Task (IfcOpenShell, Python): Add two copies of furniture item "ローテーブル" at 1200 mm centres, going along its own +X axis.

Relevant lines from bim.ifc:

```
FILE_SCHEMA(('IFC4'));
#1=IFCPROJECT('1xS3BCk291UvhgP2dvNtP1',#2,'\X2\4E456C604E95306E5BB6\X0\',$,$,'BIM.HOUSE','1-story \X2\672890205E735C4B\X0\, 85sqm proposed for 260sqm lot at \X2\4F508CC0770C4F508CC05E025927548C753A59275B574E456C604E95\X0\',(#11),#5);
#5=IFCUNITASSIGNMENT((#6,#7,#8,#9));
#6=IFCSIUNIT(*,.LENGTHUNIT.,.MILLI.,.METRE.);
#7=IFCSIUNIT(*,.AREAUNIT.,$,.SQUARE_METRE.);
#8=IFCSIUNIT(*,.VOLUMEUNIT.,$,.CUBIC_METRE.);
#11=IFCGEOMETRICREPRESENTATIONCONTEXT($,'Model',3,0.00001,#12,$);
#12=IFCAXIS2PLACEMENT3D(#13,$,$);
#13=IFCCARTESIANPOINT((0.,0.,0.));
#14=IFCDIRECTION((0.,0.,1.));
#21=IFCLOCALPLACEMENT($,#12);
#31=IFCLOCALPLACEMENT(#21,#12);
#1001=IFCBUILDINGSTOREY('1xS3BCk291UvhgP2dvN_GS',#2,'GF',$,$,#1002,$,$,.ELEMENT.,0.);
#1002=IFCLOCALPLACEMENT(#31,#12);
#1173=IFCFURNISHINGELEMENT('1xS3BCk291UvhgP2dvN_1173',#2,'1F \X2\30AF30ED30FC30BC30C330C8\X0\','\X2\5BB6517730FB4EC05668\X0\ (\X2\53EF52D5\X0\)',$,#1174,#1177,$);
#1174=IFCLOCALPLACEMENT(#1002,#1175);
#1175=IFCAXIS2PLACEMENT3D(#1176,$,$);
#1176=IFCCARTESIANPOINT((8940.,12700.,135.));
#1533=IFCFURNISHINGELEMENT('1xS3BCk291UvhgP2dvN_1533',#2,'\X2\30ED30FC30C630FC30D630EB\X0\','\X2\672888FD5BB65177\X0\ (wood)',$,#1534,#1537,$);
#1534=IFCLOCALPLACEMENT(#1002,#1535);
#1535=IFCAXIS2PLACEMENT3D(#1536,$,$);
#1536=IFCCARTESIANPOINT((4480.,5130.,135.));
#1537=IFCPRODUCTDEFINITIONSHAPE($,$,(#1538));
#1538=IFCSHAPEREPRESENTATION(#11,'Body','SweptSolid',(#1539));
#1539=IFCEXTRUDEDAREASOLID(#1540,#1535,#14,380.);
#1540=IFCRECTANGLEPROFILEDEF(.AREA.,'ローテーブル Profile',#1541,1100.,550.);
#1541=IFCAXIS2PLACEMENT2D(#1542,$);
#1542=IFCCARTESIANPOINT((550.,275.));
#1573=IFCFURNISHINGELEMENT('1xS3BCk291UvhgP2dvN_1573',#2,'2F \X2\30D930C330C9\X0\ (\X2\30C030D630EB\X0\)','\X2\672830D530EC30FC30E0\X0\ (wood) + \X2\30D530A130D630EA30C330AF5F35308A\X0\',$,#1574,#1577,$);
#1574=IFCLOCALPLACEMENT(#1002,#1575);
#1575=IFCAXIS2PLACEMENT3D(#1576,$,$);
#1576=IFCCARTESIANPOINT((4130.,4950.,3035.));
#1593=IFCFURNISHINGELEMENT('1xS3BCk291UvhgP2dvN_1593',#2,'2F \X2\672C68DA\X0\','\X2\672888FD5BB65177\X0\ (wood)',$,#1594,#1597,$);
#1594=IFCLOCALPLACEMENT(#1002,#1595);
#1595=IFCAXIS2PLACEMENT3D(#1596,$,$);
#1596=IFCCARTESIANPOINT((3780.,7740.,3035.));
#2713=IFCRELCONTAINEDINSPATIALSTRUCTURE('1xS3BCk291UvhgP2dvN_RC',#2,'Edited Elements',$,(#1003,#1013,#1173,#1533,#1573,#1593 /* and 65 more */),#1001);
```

```python
import ifcopenshell
import ifcopenshell.api.geometry
import ifcopenshell.api.root
import ifcopenshell.util.element
import ifcopenshell.util.placement
import ifcopenshell.util.unit

model = ifcopenshell.open("bim.ifc")
unit_scale = ifcopenshell.util.unit.calculate_unit_scale(model)


def reuse_history(source, copy):
    """copy_class also copies each property set's owner history, people and application; keep the originals."""
    for rel in copy.IsDefinedBy:
        if rel.is_a("IfcRelDefinesByProperties") and (history := rel.RelatingPropertyDefinition.OwnerHistory):
            rel.RelatingPropertyDefinition.OwnerHistory = source.OwnerHistory
            ifcopenshell.util.element.remove_deep2(model, history)


source = model.by_guid("1xS3BCk291UvhgP2dvN_1533")
base = ifcopenshell.util.placement.get_local_placement(source.ObjectPlacement)
step = base[:3, 0] * 1.2 / unit_scale

for i in range(1, 3):
    copy = ifcopenshell.api.root.copy_class(model, product=source)
    copy.Representation = ifcopenshell.util.element.copy_deep(
        model, source.Representation, exclude=["IfcGeometricRepresentationContext", "IfcRepresentationMap"]
    )
    reuse_history(source, copy)
    matrix = base.copy()
    matrix[:3, 3] += i * step
    print("added at", matrix[:3, 3].round(3) + 0.0)
    ifcopenshell.api.geometry.edit_object_placement(model, product=copy, matrix=matrix, is_si=False)

model.write("bim_updated.ifc")
```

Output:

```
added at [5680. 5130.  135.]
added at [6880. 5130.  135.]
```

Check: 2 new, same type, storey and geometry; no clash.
